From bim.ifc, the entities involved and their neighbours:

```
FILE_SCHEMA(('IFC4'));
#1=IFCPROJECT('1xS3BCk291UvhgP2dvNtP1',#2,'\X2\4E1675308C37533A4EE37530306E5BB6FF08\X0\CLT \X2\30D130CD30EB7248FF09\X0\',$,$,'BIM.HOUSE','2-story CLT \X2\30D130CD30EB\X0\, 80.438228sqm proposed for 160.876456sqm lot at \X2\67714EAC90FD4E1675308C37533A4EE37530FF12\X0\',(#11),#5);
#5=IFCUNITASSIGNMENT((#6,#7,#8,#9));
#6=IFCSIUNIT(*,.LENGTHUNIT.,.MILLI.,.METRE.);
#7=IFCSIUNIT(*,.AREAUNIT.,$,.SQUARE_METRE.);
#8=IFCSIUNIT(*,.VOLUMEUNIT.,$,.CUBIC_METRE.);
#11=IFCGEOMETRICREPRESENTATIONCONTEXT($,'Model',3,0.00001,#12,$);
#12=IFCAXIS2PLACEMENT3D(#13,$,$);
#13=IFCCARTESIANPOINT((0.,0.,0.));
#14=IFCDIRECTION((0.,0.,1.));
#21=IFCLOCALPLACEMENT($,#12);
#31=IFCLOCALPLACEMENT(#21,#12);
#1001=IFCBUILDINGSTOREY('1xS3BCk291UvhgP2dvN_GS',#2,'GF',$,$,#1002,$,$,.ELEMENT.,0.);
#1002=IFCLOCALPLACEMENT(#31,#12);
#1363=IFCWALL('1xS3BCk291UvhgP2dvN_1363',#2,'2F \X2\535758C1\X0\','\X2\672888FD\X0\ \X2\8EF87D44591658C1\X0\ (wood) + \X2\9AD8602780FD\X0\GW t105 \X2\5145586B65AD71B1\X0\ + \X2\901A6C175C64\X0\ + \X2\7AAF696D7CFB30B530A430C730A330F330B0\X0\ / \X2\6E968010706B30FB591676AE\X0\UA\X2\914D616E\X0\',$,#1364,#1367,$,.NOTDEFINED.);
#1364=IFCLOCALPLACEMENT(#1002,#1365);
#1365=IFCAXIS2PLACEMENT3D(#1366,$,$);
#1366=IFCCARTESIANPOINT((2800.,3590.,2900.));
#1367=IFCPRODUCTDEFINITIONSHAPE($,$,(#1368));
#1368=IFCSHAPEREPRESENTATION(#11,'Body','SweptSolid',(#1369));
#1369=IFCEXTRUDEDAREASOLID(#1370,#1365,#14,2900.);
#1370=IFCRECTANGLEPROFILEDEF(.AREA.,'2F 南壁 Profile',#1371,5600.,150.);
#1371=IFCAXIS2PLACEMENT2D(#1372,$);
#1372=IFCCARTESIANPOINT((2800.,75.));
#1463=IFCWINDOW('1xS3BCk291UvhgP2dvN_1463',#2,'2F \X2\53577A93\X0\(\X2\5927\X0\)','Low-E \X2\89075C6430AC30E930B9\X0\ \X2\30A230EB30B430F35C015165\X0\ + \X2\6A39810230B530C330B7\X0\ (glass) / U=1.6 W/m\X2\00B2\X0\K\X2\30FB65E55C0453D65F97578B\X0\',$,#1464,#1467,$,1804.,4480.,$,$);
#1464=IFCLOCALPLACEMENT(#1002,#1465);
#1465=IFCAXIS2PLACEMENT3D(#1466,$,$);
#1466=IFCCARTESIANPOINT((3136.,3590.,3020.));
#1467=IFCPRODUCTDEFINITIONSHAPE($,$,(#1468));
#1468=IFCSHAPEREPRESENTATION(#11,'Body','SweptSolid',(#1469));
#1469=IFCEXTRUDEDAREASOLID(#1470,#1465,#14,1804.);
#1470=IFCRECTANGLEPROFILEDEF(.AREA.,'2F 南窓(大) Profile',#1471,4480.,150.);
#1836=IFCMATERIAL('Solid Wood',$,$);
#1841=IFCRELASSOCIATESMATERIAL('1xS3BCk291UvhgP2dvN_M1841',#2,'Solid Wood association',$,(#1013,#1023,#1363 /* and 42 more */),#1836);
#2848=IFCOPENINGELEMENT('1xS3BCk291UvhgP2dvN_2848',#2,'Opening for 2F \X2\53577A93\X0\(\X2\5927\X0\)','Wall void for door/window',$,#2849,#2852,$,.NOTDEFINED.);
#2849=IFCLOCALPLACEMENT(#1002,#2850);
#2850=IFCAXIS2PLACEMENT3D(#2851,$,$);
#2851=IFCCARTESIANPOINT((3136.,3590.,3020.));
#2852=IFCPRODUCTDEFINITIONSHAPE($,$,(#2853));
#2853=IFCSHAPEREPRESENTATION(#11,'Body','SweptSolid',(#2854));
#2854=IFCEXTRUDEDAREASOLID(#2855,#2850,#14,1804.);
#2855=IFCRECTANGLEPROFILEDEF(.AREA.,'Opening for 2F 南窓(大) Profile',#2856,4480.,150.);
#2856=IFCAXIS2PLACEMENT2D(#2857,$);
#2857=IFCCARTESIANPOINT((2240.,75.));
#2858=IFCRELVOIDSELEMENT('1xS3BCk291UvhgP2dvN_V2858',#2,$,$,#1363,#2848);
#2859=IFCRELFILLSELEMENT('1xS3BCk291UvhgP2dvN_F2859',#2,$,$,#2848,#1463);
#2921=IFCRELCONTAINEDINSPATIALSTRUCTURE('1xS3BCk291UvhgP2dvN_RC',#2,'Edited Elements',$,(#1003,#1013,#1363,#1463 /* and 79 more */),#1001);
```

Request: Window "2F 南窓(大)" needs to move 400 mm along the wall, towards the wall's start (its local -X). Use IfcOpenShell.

```python
import ifcopenshell
import ifcopenshell.api.geometry
import ifcopenshell.util.placement
import ifcopenshell.util.unit

model = ifcopenshell.open("bim.ifc")
unit_scale = ifcopenshell.util.unit.calculate_unit_scale(model)

window = model.by_guid("1xS3BCk291UvhgP2dvN_1463")
opening = window.FillsVoids[0].RelatingOpeningElement
wall = opening.VoidsElements[0].RelatingBuildingElement

wall_matrix = ifcopenshell.util.placement.get_local_placement(wall.ObjectPlacement)
shift = wall_matrix[:3, 0] * -0.4 / unit_scale
before = ifcopenshell.util.placement.get_local_placement(window.ObjectPlacement)[:3, 3].copy()

# The window is not placed relative to its opening, so move both.
for product in (opening, window):
    matrix = ifcopenshell.util.placement.get_local_placement(product.ObjectPlacement)
    matrix[:3, 3] += shift
    ifcopenshell.api.geometry.edit_object_placement(model, product=product, matrix=matrix, is_si=False)

after = ifcopenshell.util.placement.get_local_placement(window.ObjectPlacement)[:3, 3]
print("window moved by", (after - before).round(3) + 0.0)

model.write("bim_v2.ifc")
```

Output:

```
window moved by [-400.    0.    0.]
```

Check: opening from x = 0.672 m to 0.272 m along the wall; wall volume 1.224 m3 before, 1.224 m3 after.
